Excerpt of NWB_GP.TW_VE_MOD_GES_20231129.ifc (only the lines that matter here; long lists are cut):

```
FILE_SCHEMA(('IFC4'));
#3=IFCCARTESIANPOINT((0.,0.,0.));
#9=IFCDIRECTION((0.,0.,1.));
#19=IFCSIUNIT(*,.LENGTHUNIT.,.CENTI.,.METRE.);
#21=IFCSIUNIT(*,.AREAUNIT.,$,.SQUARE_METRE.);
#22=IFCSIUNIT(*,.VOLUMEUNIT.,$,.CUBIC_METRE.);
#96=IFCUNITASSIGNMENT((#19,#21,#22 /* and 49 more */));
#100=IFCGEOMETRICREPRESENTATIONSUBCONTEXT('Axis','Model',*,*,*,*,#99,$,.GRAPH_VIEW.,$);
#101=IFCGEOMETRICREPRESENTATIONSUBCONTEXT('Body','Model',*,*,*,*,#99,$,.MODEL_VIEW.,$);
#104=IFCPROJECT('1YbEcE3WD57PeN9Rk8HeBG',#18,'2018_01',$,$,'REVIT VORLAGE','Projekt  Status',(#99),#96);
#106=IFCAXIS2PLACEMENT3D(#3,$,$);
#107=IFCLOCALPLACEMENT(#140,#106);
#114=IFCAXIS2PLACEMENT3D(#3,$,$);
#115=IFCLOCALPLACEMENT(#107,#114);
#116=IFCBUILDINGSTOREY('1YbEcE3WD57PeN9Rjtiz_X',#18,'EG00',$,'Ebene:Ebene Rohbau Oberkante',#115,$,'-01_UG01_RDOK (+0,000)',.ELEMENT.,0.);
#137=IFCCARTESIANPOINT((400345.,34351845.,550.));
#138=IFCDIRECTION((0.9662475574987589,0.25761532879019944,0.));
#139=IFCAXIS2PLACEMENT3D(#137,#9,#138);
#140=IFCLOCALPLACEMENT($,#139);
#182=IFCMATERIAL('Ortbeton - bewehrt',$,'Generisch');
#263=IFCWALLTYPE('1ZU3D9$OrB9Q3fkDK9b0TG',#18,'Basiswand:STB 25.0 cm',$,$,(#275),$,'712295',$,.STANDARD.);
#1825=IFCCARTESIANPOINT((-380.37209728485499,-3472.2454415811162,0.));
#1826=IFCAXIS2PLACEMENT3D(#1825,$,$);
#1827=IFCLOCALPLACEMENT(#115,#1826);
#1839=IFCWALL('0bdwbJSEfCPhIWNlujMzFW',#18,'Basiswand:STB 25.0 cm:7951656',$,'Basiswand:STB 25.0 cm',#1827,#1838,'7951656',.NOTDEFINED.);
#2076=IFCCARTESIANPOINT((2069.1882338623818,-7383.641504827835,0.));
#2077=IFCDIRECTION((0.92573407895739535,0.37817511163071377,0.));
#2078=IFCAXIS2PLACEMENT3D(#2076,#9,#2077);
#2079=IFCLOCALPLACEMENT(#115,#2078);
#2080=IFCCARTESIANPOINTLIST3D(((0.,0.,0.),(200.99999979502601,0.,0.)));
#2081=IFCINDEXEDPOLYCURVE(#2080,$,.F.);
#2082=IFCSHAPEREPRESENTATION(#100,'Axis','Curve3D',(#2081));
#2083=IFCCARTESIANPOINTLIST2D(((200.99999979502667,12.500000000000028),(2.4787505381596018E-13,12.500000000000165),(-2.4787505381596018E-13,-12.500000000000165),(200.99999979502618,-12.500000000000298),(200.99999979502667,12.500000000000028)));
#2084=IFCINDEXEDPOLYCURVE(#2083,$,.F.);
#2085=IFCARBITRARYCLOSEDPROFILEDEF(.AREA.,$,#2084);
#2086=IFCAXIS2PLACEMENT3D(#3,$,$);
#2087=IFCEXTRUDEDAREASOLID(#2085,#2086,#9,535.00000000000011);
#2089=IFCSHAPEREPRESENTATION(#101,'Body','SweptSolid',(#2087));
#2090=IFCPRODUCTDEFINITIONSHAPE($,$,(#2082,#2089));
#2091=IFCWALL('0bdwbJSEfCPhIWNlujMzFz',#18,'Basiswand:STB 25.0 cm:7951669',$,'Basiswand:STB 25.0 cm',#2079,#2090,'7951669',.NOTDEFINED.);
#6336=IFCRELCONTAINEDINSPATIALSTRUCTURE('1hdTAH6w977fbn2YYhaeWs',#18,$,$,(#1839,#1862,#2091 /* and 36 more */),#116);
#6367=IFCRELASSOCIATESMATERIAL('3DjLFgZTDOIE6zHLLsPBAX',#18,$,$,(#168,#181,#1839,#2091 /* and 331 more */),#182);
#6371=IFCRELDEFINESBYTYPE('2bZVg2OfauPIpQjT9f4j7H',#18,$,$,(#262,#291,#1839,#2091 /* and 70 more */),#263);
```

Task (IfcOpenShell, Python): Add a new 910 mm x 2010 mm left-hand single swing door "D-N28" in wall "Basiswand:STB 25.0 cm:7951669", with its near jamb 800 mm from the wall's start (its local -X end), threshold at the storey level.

```python
import numpy as np
import ifcopenshell
import ifcopenshell.api.feature
import ifcopenshell.api.geometry
import ifcopenshell.api.root
import ifcopenshell.api.spatial
import ifcopenshell.geom
import ifcopenshell.util.element
import ifcopenshell.util.placement
import ifcopenshell.util.representation
import ifcopenshell.util.shape
import ifcopenshell.util.unit

model = ifcopenshell.open("NWB_GP.TW_VE_MOD_GES_20231129.ifc")
unit_scale = ifcopenshell.util.unit.calculate_unit_scale(model)
settings = ifcopenshell.geom.settings()


def volume(element):
    """Net volume in cubic metres, openings subtracted."""
    shape = ifcopenshell.geom.create_shape(settings, element)
    return ifcopenshell.util.shape.get_volume(shape.geometry)


wall = model.by_guid("0bdwbJSEfCPhIWNlujMzFz")
storey = ifcopenshell.util.element.get_container(wall, ifc_class="IfcBuildingStorey")
context = ifcopenshell.util.representation.get_context(model, "Model", "Body", "MODEL_VIEW")
before = volume(wall)

width, height, from_end, sill = 0.91, 2.01, 0.8, 0.0  # metres

# The wall runs along its own X axis, and the end named is its -X end.
wall_shape = ifcopenshell.geom.create_shape(settings, wall)
x, y, z = ifcopenshell.util.shape.get_vertices(wall_shape.geometry).T
start = x.min() + from_end
face, thickness = float(y.min()), float(y.max() - y.min())
wall_matrix = ifcopenshell.util.placement.get_local_placement(wall.ObjectPlacement)
level = ifcopenshell.util.placement.get_local_placement(storey.ObjectPlacement)[2, 3]


def in_wall(x, y):
    """Placement at x, y metres in the wall's axes, at sill height."""
    matrix = wall_matrix.copy()
    matrix[:, 3] = wall_matrix @ np.array([x / unit_scale, y / unit_scale, 0.0, 1.0])
    matrix[2, 3] = level + sill / unit_scale
    return matrix


# Opening: a box that overshoots both wall faces by 50 mm.
opening = ifcopenshell.api.root.create_entity(model, ifc_class="IfcOpeningElement", predefined_type="OPENING")
box = ifcopenshell.api.geometry.add_wall_representation(
    model, context=context, length=width, height=height, thickness=thickness + 0.1
)
ifcopenshell.api.geometry.assign_representation(model, product=opening, representation=box)
ifcopenshell.api.geometry.edit_object_placement(model, product=opening, matrix=in_wall(start, face - 0.05), is_si=False)
ifcopenshell.api.feature.add_feature(model, feature=opening, element=wall)

door = ifcopenshell.api.root.create_entity(model, ifc_class="IfcDoor", name="D-N28", predefined_type="DOOR")
door.OverallWidth, door.OverallHeight = width / unit_scale, height / unit_scale
door.OperationType = "SINGLE_SWING_LEFT"
body = ifcopenshell.api.geometry.add_door_representation(
    model,
    context=context,
    overall_width=door.OverallWidth,
    overall_height=door.OverallHeight,
    operation_type="SINGLE_SWING_LEFT",
    lining_properties={"LiningDepth": thickness / unit_scale, "ThresholdDepth": thickness / unit_scale},
)
ifcopenshell.api.geometry.assign_representation(model, product=door, representation=body)
ifcopenshell.api.spatial.assign_container(model, products=[door], relating_structure=storey)
ifcopenshell.api.feature.add_filling(model, opening=opening, element=door)

# The lining spans the wall, so the door starts at the wall face.
ifcopenshell.api.geometry.edit_object_placement(model, product=door, matrix=in_wall(start, face), is_si=False)

after = volume(wall)

print(f"wall volume {before:.3f} -> {after:.3f} m3")

model.write("NWB_GP.TW_VE_MOD_GES_20231129-out.ifc")
```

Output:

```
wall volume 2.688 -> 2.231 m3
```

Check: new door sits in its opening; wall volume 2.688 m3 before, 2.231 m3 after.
